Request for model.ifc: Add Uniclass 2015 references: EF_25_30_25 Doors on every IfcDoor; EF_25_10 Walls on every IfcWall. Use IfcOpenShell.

First a look at what the model holds.

```python
import ifcopenshell

model = ifcopenshell.open("model.ifc")
print(model.schema)
print("classifications:", [c.Name for c in model.by_type("IfcClassification")])
for ifc_class in ("IfcDoor", "IfcRoof", "IfcStair", "IfcWall", "IfcWindow"):
    print(ifc_class, len(model.by_type(ifc_class)))
```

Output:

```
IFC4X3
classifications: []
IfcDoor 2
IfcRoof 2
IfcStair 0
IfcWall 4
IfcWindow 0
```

```python
import ifcopenshell
import ifcopenshell.api.classification

model = ifcopenshell.open("model.ifc")

system = ifcopenshell.api.classification.add_classification(model, classification="Uniclass 2015")

codes = {
    "IfcDoor": ("EF_25_30_25", "Doors"),
    "IfcWall": ("EF_25_10", "Walls"),
}
for ifc_class, (code, name) in codes.items():
    products = model.by_type(ifc_class)
    ifcopenshell.api.classification.add_reference(
        model, products=products, classification=system, identification=code, name=name
    )
    print(code, len(products))

model.write("model_updated.ifc")
```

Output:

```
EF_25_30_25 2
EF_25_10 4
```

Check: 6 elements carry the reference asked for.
